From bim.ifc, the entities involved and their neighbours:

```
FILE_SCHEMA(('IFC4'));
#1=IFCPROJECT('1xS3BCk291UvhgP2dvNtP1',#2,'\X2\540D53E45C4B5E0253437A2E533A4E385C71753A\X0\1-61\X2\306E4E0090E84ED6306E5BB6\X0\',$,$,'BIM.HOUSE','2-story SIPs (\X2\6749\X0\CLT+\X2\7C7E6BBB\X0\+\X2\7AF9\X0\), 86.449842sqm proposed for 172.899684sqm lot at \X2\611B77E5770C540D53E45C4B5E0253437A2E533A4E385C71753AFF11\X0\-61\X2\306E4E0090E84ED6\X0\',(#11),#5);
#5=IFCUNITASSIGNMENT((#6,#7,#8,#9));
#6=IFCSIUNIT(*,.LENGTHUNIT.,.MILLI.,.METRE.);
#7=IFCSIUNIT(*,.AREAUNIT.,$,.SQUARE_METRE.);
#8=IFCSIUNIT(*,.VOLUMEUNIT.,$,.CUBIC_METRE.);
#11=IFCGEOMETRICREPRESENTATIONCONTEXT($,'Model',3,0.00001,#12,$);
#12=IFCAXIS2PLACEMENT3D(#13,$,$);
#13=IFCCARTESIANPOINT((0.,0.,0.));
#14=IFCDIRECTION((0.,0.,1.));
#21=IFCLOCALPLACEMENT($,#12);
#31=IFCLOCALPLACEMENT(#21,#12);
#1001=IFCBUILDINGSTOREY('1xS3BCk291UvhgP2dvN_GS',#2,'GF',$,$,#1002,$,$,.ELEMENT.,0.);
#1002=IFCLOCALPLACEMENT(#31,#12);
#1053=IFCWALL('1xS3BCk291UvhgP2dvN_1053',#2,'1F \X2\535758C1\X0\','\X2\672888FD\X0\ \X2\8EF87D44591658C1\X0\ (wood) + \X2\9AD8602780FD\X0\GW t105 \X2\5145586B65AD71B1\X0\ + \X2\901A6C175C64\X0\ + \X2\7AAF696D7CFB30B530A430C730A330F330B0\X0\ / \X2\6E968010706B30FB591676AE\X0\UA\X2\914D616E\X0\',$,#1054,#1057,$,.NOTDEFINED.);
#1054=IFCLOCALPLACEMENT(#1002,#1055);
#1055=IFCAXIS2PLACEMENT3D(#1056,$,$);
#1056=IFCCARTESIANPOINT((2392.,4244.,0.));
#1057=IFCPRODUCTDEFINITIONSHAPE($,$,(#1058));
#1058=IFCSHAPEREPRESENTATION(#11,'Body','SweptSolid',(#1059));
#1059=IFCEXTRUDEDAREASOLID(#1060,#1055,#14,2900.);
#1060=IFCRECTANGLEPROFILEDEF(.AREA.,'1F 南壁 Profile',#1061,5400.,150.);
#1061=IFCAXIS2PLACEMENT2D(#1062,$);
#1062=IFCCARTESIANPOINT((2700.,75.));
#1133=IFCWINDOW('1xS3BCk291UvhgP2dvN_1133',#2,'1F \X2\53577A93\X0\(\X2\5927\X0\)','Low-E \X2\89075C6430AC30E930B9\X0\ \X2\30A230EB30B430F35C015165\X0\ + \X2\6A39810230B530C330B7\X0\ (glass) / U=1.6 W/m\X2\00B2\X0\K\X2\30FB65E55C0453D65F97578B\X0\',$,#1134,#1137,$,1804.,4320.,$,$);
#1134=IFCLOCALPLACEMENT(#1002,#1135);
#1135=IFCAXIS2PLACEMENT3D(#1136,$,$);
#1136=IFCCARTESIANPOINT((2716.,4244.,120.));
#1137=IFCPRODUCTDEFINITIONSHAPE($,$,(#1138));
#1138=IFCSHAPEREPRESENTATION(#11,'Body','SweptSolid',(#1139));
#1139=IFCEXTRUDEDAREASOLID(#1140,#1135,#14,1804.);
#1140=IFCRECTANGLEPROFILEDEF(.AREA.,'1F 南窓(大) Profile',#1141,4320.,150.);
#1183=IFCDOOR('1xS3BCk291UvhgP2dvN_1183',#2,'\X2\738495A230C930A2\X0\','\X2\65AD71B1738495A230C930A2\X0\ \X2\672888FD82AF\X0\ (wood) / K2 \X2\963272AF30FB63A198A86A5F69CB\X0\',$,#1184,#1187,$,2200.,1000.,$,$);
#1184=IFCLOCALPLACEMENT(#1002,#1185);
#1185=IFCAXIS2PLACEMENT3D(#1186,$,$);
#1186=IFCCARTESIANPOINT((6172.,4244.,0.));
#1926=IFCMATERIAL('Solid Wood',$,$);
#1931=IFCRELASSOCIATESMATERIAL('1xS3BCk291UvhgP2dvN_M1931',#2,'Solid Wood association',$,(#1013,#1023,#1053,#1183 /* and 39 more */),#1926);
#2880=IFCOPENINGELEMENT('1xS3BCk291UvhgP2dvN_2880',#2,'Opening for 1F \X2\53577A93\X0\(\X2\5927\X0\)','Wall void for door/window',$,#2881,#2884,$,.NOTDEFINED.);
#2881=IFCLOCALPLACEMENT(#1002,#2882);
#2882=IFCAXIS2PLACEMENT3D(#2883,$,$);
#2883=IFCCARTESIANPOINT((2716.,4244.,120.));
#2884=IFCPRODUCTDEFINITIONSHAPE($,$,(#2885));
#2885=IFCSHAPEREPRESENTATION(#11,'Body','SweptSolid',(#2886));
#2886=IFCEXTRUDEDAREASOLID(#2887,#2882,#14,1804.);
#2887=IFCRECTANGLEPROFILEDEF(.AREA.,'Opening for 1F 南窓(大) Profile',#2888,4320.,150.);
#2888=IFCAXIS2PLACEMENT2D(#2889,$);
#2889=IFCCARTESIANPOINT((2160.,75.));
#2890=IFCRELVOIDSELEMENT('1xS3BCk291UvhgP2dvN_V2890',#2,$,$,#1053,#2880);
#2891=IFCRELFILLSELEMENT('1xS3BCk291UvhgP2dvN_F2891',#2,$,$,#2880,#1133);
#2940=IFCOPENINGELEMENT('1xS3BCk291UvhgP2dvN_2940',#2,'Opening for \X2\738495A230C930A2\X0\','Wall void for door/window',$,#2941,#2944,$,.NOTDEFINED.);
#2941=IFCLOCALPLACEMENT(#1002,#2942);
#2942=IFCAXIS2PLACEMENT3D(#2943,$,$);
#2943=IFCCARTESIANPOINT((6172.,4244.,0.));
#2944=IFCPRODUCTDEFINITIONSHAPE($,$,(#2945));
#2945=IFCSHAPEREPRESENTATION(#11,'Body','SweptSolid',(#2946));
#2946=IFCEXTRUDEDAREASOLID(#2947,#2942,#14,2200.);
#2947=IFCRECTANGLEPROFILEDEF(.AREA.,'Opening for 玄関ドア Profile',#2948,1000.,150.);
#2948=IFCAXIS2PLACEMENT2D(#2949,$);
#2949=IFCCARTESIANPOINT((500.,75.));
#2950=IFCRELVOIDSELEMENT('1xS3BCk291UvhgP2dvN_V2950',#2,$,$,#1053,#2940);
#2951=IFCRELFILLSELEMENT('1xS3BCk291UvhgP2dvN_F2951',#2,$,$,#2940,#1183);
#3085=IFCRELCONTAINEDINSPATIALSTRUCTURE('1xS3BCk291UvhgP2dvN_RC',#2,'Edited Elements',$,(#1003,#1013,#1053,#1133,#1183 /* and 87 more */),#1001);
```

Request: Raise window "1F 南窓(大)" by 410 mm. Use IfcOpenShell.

```python
import numpy as np
import ifcopenshell
import ifcopenshell.api.geometry
import ifcopenshell.util.placement
import ifcopenshell.util.unit

model = ifcopenshell.open("bim.ifc")
unit_scale = ifcopenshell.util.unit.calculate_unit_scale(model)

window = model.by_guid("1xS3BCk291UvhgP2dvN_1133")
opening = window.FillsVoids[0].RelatingOpeningElement
dz = 0.41 / unit_scale

shift = np.array([0.0, 0.0, dz])
# The window is not placed relative to its opening, so move both.
for product in (opening, window):
    matrix = ifcopenshell.util.placement.get_local_placement(product.ObjectPlacement)
    matrix[:3, 3] += shift
    ifcopenshell.api.geometry.edit_object_placement(model, product=product, matrix=matrix, is_si=False)

print(f"moved by {dz * unit_scale:+.3f} m")

model.write("bim_v2.ifc")
```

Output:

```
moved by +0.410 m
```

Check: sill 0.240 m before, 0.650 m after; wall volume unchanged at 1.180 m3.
